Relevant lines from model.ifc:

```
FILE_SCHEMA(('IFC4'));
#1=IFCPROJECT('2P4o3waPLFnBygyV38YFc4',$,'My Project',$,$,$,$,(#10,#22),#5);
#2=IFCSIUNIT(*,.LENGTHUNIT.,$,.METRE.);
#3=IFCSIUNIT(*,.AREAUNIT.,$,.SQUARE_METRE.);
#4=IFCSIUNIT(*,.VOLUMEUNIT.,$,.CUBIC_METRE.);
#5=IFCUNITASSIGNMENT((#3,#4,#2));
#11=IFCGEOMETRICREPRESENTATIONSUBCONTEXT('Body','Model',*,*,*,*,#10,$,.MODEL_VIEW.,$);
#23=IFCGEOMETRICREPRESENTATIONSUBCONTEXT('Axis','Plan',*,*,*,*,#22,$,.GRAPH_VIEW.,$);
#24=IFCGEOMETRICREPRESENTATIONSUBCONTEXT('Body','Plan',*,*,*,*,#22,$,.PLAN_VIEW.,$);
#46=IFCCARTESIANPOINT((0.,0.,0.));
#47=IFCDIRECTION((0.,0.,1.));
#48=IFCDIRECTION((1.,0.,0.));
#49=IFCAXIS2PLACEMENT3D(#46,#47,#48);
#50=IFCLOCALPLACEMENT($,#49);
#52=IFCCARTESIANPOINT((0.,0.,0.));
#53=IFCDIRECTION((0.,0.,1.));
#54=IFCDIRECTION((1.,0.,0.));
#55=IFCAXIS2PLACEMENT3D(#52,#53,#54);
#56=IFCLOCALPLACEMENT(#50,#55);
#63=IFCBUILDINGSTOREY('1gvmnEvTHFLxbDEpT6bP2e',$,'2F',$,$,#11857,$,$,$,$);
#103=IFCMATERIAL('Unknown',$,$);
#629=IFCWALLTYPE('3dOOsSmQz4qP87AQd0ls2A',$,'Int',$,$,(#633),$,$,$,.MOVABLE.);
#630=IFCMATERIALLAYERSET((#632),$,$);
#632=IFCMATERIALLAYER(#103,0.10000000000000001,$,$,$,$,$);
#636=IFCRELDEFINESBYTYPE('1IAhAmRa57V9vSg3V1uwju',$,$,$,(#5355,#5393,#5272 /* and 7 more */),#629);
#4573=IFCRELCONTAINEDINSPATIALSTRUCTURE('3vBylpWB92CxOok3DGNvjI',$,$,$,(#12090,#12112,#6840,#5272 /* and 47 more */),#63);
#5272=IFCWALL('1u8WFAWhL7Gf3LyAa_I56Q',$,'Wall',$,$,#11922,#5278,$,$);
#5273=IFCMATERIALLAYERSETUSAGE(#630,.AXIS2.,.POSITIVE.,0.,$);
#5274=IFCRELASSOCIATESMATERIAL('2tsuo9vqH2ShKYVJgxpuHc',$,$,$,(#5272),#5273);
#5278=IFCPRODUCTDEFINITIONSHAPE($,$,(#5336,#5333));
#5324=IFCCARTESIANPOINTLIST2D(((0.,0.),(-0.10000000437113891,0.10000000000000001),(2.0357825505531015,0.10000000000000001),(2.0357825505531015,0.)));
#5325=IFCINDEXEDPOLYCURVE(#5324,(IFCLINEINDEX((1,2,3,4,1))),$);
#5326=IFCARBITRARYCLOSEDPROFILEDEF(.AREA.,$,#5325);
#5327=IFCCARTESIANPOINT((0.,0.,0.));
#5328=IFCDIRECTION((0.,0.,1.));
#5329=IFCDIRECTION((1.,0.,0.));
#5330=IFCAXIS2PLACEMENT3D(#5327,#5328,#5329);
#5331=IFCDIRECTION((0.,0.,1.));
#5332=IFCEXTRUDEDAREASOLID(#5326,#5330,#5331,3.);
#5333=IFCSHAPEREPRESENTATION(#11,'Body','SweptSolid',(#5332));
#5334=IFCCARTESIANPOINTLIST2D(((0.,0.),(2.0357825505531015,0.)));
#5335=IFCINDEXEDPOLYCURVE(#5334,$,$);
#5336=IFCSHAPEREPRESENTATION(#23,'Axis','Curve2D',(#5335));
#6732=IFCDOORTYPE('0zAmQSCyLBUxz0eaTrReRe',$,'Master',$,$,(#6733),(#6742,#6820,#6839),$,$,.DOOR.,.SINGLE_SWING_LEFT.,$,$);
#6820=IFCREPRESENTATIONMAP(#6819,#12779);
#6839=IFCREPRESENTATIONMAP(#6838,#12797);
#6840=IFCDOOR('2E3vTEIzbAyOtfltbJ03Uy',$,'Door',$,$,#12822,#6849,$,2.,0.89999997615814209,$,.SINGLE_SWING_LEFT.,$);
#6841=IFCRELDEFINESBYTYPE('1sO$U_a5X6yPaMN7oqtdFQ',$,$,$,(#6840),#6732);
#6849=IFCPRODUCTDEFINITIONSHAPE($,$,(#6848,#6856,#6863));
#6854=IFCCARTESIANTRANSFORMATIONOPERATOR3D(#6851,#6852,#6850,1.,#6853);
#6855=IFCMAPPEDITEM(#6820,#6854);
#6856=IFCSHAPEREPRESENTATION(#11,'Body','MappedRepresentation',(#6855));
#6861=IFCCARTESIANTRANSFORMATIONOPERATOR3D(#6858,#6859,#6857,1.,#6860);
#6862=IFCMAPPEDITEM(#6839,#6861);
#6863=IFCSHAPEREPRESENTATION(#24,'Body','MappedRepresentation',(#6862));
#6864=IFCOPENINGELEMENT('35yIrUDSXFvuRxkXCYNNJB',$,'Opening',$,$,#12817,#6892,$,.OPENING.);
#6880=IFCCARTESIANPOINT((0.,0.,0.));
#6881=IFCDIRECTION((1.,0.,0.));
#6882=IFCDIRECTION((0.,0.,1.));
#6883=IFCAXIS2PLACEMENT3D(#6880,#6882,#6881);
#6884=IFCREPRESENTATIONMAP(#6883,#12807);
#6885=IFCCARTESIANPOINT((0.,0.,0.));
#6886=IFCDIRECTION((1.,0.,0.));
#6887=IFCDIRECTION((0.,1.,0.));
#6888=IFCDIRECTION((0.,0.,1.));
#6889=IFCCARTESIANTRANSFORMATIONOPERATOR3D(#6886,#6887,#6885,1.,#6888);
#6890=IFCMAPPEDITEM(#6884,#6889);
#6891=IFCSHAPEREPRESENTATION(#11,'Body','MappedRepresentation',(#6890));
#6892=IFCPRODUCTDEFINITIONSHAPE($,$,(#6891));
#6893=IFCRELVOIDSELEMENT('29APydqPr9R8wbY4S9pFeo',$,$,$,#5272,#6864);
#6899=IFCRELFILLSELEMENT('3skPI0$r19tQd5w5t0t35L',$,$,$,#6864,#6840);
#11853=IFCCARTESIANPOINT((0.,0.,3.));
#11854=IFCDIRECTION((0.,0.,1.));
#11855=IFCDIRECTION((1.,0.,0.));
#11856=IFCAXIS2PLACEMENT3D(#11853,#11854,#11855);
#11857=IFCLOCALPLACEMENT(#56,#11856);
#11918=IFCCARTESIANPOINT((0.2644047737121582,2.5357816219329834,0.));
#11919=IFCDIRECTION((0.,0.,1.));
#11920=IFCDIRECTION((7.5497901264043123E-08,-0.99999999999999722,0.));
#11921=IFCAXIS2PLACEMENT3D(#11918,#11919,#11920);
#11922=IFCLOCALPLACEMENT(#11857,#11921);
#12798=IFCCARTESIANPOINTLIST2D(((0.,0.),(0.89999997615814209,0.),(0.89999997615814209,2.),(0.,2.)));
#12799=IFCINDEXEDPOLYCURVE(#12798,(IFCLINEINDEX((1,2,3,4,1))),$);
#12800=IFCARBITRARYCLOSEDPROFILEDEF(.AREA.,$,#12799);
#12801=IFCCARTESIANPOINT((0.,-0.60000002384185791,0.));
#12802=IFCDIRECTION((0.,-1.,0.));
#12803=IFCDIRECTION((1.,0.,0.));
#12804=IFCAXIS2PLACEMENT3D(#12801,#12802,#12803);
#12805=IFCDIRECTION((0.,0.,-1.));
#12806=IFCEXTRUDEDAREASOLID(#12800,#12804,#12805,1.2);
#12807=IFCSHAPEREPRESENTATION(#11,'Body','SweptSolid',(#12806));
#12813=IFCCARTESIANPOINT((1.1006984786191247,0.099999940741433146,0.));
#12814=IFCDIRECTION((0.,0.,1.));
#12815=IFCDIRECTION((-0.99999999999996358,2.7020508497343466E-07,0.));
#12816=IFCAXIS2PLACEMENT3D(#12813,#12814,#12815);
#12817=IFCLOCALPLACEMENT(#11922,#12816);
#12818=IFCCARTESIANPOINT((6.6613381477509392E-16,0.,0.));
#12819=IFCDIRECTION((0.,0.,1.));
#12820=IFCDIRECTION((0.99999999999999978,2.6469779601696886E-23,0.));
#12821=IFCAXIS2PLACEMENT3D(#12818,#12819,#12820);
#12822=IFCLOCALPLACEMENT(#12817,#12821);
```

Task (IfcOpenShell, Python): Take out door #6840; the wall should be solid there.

```python
import ifcopenshell
import ifcopenshell.api.feature
import ifcopenshell.api.root
import ifcopenshell.geom
import ifcopenshell.util.shape

model = ifcopenshell.open("model.ifc")
settings = ifcopenshell.geom.settings()


def volume(element):
    """Net volume in cubic metres, openings subtracted."""
    shape = ifcopenshell.geom.create_shape(settings, element)
    return ifcopenshell.util.shape.get_volume(shape.geometry)


door = model.by_id(6840)
opening = door.FillsVoids[0].RelatingOpeningElement
wall = opening.VoidsElements[0].RelatingBuildingElement
before = volume(wall)

ifcopenshell.api.root.remove_product(model, product=door)
ifcopenshell.api.feature.remove_feature(model, feature=opening)

after = volume(wall)

print(f"wall volume {before:.3f} -> {after:.3f} m3")

model.write("model_updated.ifc")
```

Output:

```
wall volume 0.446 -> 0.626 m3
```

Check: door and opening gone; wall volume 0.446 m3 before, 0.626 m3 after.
